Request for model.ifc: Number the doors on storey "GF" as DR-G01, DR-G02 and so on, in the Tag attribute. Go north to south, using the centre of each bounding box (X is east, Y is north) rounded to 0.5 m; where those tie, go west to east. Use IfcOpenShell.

First a look at what the model holds.

```python
import ifcopenshell
import ifcopenshell.util.element
import ifcopenshell.util.placement

model = ifcopenshell.open("model.ifc")
print(model.schema)
storey = next(s for s in model.by_type("IfcBuildingStorey") if s.Name == "GF")
doors = [e for e in ifcopenshell.util.element.get_decomposition(storey) if e.is_a("IfcDoor")]
for e in sorted(doors, key=lambda e: e.id()):
    origin = ifcopenshell.util.placement.get_local_placement(e.ObjectPlacement)[:3, 3]
    print(e.id(), e.Tag, e.Name, origin.round(2) + 0.0, sep=" | ")
```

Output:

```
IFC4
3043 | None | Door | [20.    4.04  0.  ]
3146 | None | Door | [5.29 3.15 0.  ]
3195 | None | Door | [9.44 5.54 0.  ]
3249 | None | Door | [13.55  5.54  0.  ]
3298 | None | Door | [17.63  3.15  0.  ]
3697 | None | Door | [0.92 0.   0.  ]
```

```python
import ifcopenshell
import ifcopenshell.geom
import ifcopenshell.util.element
import ifcopenshell.util.shape

model = ifcopenshell.open("model.ifc")
settings = ifcopenshell.geom.settings()
settings.set("use-world-coords", True)


def centre(element):
    shape = ifcopenshell.geom.create_shape(settings, element)
    return ifcopenshell.util.shape.get_bbox_centroid(shape.geometry)


storey = next(s for s in model.by_type("IfcBuildingStorey") if s.Name == "GF")
doors = [e for e in ifcopenshell.util.element.get_decomposition(storey) if e.is_a("IfcDoor")]

# Insertion points can sit at a corner or the storey origin, so sort by the geometry (in metres).
centres = {e: centre(e) for e in doors}
doors.sort(key=lambda e: (-round(centres[e][1] / 0.5), centres[e][0]))

for i, e in enumerate(doors, start=1):
    number = f"DR-G{i:02d}"
    e.Tag = number
    print(e.id(), number)

model.write("model_updated.ifc")
```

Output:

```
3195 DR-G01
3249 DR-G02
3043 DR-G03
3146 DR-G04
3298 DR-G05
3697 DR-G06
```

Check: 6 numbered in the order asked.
